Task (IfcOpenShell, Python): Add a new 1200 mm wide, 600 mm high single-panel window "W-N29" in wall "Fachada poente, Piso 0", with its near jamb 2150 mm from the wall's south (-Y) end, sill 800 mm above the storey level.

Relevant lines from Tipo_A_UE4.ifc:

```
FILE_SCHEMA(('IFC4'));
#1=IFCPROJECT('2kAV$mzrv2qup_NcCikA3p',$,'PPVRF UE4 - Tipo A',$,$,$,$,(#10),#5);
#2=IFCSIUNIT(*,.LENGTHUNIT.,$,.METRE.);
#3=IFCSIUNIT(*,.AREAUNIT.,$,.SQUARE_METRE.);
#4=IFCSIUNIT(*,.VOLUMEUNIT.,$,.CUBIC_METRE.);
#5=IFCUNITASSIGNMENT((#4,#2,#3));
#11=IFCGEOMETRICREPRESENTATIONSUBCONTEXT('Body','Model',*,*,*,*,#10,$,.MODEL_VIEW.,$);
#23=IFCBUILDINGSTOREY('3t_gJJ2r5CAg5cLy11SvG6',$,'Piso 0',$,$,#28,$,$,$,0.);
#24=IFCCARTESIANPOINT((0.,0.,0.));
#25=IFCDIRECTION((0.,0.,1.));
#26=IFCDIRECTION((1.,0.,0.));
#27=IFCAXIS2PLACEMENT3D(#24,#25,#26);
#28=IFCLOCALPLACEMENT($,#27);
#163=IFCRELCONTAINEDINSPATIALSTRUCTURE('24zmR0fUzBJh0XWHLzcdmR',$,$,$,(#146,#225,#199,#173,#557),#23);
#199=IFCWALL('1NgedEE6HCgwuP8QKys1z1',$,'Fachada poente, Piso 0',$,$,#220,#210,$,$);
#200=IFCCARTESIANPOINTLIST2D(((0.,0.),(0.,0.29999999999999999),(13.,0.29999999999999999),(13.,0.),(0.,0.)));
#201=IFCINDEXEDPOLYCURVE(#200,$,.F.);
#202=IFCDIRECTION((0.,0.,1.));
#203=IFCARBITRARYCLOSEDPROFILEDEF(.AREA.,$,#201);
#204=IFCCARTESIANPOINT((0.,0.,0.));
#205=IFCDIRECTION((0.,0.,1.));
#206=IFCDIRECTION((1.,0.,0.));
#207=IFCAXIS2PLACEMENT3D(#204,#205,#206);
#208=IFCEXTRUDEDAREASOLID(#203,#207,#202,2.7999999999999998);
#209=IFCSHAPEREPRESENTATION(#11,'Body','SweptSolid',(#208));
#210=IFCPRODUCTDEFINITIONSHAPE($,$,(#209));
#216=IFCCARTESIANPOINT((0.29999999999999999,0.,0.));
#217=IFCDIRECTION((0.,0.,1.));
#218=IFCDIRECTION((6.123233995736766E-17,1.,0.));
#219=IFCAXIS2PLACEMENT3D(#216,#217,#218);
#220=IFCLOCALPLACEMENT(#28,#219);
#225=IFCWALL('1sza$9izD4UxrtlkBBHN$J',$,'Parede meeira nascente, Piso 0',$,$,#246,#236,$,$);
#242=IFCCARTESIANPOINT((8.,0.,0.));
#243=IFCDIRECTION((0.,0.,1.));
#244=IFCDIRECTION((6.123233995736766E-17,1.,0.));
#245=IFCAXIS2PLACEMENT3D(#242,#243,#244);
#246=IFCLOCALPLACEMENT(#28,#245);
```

```python
import numpy as np
import ifcopenshell
import ifcopenshell.api.feature
import ifcopenshell.api.geometry
import ifcopenshell.api.root
import ifcopenshell.api.spatial
import ifcopenshell.geom
import ifcopenshell.util.element
import ifcopenshell.util.placement
import ifcopenshell.util.representation
import ifcopenshell.util.shape
import ifcopenshell.util.unit

model = ifcopenshell.open("Tipo_A_UE4.ifc")
unit_scale = ifcopenshell.util.unit.calculate_unit_scale(model)
settings = ifcopenshell.geom.settings()


def volume(element):
    """Net volume in cubic metres, openings subtracted."""
    shape = ifcopenshell.geom.create_shape(settings, element)
    return ifcopenshell.util.shape.get_volume(shape.geometry)


wall = model.by_guid("1NgedEE6HCgwuP8QKys1z1")
storey = ifcopenshell.util.element.get_container(wall, ifc_class="IfcBuildingStorey")
context = ifcopenshell.util.representation.get_context(model, "Model", "Body", "MODEL_VIEW")
before = volume(wall)

width, height, from_end, sill = 1.2, 0.6, 2.15, 0.8  # metres

# The wall runs along its own X axis, and the end named is its -X end.
wall_shape = ifcopenshell.geom.create_shape(settings, wall)
x, y, z = ifcopenshell.util.shape.get_vertices(wall_shape.geometry).T
start = x.min() + from_end
face, thickness = float(y.min()), float(y.max() - y.min())
wall_matrix = ifcopenshell.util.placement.get_local_placement(wall.ObjectPlacement)
level = ifcopenshell.util.placement.get_local_placement(storey.ObjectPlacement)[2, 3]


def in_wall(x, y):
    """Placement at x, y metres in the wall's axes, at sill height."""
    matrix = wall_matrix.copy()
    matrix[:, 3] = wall_matrix @ np.array([x / unit_scale, y / unit_scale, 0.0, 1.0])
    matrix[2, 3] = level + sill / unit_scale
    return matrix


# Opening: a box that overshoots both wall faces by 50 mm.
opening = ifcopenshell.api.root.create_entity(model, ifc_class="IfcOpeningElement", predefined_type="OPENING")
box = ifcopenshell.api.geometry.add_wall_representation(
    model, context=context, length=width, height=height, thickness=thickness + 0.1
)
ifcopenshell.api.geometry.assign_representation(model, product=opening, representation=box)
ifcopenshell.api.geometry.edit_object_placement(model, product=opening, matrix=in_wall(start, face - 0.05), is_si=False)
ifcopenshell.api.feature.add_feature(model, feature=opening, element=wall)

window = ifcopenshell.api.root.create_entity(model, ifc_class="IfcWindow", name="W-N29", predefined_type="WINDOW")
window.OverallWidth, window.OverallHeight = width / unit_scale, height / unit_scale
window.PartitioningType = "SINGLE_PANEL"
body = ifcopenshell.api.geometry.add_window_representation(
    model,
    context=context,
    overall_width=window.OverallWidth,
    overall_height=window.OverallHeight,
    partition_type="SINGLE_PANEL",
)
ifcopenshell.api.geometry.assign_representation(model, product=window, representation=body)
ifcopenshell.api.spatial.assign_container(model, products=[window], relating_structure=storey)
ifcopenshell.api.feature.add_filling(model, opening=opening, element=window)

# Centre the window in the wall's thickness.
ifcopenshell.api.geometry.edit_object_placement(model, product=window, matrix=in_wall(start, face), is_si=False)
window_shape = ifcopenshell.geom.create_shape(settings, window)
depth = ifcopenshell.util.shape.get_vertices(window_shape.geometry)[:, 1]
offset = face + thickness / 2 - (depth.min() + depth.max()) / 2
ifcopenshell.api.geometry.edit_object_placement(model, product=window, matrix=in_wall(start, offset), is_si=False)

after = volume(wall)

print(f"wall volume {before:.3f} -> {after:.3f} m3")

model.write("Tipo_A_UE4_v2.ifc")
```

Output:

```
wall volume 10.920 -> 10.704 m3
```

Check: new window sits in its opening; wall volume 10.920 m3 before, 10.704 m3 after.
